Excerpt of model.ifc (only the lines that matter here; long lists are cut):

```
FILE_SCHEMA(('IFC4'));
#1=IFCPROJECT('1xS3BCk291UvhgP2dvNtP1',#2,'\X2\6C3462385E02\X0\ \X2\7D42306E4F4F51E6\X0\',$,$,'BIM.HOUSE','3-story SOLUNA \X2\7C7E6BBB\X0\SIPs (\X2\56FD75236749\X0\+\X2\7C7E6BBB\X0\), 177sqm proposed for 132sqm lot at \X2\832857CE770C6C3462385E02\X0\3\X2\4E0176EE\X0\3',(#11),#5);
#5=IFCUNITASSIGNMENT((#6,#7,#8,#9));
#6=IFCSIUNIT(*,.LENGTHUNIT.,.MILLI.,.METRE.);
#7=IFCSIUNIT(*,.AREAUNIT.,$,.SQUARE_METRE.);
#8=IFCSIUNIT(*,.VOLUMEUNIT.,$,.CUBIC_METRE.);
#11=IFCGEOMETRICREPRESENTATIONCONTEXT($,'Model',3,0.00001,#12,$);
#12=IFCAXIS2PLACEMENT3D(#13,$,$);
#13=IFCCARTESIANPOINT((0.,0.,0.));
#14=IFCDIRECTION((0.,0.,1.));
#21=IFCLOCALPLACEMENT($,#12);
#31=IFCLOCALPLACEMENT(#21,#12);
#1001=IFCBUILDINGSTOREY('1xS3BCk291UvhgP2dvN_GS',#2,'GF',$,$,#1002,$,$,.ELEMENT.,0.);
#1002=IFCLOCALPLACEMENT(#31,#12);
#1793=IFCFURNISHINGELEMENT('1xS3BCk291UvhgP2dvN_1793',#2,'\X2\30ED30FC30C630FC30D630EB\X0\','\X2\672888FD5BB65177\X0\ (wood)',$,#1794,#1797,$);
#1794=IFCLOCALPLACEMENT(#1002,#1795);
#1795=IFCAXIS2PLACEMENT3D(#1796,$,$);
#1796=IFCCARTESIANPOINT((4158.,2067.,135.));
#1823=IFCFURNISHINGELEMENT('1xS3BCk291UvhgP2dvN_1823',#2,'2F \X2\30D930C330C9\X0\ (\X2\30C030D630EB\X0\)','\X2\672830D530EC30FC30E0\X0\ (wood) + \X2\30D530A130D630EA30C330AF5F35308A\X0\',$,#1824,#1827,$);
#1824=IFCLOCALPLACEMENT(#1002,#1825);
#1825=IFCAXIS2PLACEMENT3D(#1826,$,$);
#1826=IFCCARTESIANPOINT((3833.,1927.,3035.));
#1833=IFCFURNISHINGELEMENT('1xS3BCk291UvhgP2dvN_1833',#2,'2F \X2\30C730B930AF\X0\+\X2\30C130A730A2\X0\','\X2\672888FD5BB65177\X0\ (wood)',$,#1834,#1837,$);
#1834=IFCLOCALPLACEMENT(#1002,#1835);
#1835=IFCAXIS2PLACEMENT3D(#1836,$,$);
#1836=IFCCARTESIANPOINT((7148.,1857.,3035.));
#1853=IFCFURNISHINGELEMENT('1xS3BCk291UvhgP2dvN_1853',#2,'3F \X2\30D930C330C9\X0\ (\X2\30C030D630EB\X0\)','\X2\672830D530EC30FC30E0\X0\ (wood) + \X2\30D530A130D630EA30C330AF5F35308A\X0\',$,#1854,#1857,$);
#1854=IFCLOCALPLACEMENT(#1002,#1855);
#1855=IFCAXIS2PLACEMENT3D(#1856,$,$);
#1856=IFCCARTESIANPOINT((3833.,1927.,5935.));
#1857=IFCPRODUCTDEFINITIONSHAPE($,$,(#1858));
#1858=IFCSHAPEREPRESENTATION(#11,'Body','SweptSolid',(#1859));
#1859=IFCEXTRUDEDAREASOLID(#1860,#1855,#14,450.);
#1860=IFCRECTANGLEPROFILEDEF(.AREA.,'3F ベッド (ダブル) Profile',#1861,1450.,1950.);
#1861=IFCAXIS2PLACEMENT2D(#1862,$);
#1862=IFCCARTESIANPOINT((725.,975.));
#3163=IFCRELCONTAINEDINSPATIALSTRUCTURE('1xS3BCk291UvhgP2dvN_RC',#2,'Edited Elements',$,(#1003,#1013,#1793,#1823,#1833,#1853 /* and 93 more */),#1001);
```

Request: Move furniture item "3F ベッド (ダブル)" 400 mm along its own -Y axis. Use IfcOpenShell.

```python
import ifcopenshell
import ifcopenshell.api.geometry
import ifcopenshell.util.placement
import ifcopenshell.util.unit

model = ifcopenshell.open("model.ifc")
unit_scale = ifcopenshell.util.unit.calculate_unit_scale(model)

item = model.by_id(1853)
matrix = ifcopenshell.util.placement.get_local_placement(item.ObjectPlacement)
matrix[:3, 3] -= matrix[:3, 1] * 0.4 / unit_scale
ifcopenshell.api.geometry.edit_object_placement(model, product=item, matrix=matrix, is_si=False)

print(ifcopenshell.util.placement.get_local_placement(item.ObjectPlacement).round(3) + 0.0)

model.write("model-out.ifc")
```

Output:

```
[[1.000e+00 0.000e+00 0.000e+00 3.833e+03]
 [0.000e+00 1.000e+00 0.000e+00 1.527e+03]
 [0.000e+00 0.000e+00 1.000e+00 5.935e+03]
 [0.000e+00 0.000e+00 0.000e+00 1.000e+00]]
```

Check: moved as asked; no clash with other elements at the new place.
